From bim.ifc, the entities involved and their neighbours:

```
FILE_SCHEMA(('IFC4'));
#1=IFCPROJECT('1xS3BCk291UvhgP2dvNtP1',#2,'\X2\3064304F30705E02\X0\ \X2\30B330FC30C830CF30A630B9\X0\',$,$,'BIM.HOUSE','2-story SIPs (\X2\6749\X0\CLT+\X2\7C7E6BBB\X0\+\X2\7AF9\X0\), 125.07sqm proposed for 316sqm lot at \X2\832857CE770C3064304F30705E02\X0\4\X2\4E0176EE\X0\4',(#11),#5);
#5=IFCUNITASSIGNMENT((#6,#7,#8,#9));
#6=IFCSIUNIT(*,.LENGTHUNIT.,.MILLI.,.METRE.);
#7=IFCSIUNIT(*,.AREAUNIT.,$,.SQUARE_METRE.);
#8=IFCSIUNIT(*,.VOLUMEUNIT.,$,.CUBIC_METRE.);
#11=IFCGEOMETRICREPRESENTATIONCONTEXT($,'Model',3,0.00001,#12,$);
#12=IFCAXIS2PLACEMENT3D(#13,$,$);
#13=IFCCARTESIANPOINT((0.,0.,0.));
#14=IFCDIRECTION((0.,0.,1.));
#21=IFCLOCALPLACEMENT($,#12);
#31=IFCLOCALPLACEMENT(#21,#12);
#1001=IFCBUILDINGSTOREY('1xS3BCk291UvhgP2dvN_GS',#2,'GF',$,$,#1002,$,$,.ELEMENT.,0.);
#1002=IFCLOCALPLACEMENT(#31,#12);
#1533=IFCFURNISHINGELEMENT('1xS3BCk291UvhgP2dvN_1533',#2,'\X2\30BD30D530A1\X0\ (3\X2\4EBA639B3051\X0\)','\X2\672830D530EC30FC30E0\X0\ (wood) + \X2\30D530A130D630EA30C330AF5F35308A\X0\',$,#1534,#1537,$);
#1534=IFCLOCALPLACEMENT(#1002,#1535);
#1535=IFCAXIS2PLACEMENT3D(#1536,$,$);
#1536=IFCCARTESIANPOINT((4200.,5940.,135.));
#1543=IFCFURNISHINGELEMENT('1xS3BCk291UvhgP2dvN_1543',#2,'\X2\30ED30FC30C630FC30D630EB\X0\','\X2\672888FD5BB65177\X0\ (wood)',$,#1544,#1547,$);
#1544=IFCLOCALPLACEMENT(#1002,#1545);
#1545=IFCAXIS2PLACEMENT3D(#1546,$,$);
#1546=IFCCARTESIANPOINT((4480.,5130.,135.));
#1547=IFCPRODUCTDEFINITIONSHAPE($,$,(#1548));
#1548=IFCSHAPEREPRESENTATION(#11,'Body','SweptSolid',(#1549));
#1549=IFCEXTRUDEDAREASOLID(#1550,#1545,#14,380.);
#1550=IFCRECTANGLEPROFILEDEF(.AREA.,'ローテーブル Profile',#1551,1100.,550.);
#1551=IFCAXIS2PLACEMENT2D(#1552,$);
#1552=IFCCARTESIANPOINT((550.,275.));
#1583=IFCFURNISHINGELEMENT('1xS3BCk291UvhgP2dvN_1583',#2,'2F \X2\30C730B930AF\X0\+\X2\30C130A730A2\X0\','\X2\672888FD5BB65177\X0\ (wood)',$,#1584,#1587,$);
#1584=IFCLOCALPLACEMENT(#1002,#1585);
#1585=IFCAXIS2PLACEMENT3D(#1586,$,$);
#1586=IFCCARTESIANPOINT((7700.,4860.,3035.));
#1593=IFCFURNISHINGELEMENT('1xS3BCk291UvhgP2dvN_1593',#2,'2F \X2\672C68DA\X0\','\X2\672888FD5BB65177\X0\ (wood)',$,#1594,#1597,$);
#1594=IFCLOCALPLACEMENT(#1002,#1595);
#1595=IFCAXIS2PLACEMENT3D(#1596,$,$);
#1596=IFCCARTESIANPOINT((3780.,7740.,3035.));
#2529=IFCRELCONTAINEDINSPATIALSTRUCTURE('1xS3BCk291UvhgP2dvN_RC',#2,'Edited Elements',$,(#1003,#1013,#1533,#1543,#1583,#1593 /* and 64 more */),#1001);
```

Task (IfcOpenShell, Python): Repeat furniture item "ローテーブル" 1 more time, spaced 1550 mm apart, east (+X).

```python
import numpy as np
import ifcopenshell
import ifcopenshell.api.geometry
import ifcopenshell.api.root
import ifcopenshell.util.element
import ifcopenshell.util.placement

model = ifcopenshell.open("bim.ifc")


def reuse_history(source, copy):
    """copy_class also copies each property set's owner history, people and application; keep the originals."""
    for rel in copy.IsDefinedBy:
        if rel.is_a("IfcRelDefinesByProperties") and (history := rel.RelatingPropertyDefinition.OwnerHistory):
            rel.RelatingPropertyDefinition.OwnerHistory = source.OwnerHistory
            ifcopenshell.util.element.remove_deep2(model, history)


source = model.by_id(1543)
base = ifcopenshell.util.placement.get_local_placement(source.ObjectPlacement)
step = np.array([1.0, 0.0, 0.0]) * 1550.0

for i in range(1, 2):
    copy = ifcopenshell.api.root.copy_class(model, product=source)
    copy.Representation = ifcopenshell.util.element.copy_deep(
        model, source.Representation, exclude=["IfcGeometricRepresentationContext", "IfcRepresentationMap"]
    )
    reuse_history(source, copy)
    matrix = base.copy()
    matrix[:3, 3] += i * step
    print("added at", matrix[:3, 3].round(3) + 0.0)
    ifcopenshell.api.geometry.edit_object_placement(model, product=copy, matrix=matrix, is_si=False)

model.write("bim_edited.ifc")
```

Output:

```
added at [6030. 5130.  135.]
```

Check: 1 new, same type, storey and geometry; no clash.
